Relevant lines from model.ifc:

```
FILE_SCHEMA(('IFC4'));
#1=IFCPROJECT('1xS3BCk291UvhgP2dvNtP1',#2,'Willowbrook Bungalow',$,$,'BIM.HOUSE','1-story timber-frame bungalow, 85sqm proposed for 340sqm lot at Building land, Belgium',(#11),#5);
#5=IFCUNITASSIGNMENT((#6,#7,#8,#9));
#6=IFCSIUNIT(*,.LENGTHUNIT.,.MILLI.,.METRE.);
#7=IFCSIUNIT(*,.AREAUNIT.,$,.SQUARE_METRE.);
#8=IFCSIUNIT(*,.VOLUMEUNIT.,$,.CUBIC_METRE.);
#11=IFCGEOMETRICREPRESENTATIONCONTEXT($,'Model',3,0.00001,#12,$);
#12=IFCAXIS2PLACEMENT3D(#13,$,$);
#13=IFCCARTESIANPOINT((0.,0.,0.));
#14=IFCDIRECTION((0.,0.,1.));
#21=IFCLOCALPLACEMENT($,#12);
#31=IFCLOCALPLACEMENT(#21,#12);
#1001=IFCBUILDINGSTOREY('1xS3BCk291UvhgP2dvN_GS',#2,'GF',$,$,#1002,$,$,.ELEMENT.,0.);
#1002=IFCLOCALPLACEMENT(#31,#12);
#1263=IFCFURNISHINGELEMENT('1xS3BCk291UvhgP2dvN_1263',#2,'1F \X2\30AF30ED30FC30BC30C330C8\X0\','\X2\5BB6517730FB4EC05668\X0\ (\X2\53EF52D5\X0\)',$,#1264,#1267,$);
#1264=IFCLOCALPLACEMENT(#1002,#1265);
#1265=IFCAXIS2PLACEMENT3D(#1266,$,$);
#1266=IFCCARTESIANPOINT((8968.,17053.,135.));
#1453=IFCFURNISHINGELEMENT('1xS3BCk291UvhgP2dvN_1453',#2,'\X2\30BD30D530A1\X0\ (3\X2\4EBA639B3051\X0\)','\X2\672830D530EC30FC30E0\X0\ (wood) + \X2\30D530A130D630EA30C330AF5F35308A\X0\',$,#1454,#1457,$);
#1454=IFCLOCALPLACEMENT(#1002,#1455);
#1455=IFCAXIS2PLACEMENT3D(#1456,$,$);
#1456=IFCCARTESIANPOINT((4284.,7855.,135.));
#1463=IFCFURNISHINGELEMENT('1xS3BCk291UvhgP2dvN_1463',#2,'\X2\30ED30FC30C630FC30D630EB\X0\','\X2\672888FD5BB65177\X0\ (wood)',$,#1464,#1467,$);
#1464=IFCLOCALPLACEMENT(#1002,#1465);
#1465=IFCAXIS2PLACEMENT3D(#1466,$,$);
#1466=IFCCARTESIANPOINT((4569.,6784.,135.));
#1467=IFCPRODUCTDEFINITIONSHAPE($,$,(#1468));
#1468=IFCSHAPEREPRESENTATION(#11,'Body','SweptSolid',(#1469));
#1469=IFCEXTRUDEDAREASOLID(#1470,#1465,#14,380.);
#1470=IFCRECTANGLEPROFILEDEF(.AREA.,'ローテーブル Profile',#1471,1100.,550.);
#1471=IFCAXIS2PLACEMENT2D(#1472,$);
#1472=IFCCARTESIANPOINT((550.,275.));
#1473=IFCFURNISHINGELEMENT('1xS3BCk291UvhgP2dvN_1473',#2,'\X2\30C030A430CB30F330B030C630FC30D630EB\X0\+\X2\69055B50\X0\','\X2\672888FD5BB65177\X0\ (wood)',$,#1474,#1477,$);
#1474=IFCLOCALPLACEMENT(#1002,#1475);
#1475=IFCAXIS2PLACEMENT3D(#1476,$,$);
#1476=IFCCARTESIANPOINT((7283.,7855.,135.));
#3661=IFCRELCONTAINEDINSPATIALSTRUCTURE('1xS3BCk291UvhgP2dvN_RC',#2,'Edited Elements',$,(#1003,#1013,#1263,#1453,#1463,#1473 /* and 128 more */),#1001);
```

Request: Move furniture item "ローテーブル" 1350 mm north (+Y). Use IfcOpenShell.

```python
import ifcopenshell
import ifcopenshell.api.geometry
import ifcopenshell.util.placement
import ifcopenshell.util.unit

model = ifcopenshell.open("model.ifc")
unit_scale = ifcopenshell.util.unit.calculate_unit_scale(model)

item = model.by_guid("1xS3BCk291UvhgP2dvN_1463")
matrix = ifcopenshell.util.placement.get_local_placement(item.ObjectPlacement)
matrix[1, 3] += 1.35 / unit_scale
ifcopenshell.api.geometry.edit_object_placement(model, product=item, matrix=matrix, is_si=False)

print(ifcopenshell.util.placement.get_local_placement(item.ObjectPlacement).round(3) + 0.0)

model.write("model-out.ifc")
```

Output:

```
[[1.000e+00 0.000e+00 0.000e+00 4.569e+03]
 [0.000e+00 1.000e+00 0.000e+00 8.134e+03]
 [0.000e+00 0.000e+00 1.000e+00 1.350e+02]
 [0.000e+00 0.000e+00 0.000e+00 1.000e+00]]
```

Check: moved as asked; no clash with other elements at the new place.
